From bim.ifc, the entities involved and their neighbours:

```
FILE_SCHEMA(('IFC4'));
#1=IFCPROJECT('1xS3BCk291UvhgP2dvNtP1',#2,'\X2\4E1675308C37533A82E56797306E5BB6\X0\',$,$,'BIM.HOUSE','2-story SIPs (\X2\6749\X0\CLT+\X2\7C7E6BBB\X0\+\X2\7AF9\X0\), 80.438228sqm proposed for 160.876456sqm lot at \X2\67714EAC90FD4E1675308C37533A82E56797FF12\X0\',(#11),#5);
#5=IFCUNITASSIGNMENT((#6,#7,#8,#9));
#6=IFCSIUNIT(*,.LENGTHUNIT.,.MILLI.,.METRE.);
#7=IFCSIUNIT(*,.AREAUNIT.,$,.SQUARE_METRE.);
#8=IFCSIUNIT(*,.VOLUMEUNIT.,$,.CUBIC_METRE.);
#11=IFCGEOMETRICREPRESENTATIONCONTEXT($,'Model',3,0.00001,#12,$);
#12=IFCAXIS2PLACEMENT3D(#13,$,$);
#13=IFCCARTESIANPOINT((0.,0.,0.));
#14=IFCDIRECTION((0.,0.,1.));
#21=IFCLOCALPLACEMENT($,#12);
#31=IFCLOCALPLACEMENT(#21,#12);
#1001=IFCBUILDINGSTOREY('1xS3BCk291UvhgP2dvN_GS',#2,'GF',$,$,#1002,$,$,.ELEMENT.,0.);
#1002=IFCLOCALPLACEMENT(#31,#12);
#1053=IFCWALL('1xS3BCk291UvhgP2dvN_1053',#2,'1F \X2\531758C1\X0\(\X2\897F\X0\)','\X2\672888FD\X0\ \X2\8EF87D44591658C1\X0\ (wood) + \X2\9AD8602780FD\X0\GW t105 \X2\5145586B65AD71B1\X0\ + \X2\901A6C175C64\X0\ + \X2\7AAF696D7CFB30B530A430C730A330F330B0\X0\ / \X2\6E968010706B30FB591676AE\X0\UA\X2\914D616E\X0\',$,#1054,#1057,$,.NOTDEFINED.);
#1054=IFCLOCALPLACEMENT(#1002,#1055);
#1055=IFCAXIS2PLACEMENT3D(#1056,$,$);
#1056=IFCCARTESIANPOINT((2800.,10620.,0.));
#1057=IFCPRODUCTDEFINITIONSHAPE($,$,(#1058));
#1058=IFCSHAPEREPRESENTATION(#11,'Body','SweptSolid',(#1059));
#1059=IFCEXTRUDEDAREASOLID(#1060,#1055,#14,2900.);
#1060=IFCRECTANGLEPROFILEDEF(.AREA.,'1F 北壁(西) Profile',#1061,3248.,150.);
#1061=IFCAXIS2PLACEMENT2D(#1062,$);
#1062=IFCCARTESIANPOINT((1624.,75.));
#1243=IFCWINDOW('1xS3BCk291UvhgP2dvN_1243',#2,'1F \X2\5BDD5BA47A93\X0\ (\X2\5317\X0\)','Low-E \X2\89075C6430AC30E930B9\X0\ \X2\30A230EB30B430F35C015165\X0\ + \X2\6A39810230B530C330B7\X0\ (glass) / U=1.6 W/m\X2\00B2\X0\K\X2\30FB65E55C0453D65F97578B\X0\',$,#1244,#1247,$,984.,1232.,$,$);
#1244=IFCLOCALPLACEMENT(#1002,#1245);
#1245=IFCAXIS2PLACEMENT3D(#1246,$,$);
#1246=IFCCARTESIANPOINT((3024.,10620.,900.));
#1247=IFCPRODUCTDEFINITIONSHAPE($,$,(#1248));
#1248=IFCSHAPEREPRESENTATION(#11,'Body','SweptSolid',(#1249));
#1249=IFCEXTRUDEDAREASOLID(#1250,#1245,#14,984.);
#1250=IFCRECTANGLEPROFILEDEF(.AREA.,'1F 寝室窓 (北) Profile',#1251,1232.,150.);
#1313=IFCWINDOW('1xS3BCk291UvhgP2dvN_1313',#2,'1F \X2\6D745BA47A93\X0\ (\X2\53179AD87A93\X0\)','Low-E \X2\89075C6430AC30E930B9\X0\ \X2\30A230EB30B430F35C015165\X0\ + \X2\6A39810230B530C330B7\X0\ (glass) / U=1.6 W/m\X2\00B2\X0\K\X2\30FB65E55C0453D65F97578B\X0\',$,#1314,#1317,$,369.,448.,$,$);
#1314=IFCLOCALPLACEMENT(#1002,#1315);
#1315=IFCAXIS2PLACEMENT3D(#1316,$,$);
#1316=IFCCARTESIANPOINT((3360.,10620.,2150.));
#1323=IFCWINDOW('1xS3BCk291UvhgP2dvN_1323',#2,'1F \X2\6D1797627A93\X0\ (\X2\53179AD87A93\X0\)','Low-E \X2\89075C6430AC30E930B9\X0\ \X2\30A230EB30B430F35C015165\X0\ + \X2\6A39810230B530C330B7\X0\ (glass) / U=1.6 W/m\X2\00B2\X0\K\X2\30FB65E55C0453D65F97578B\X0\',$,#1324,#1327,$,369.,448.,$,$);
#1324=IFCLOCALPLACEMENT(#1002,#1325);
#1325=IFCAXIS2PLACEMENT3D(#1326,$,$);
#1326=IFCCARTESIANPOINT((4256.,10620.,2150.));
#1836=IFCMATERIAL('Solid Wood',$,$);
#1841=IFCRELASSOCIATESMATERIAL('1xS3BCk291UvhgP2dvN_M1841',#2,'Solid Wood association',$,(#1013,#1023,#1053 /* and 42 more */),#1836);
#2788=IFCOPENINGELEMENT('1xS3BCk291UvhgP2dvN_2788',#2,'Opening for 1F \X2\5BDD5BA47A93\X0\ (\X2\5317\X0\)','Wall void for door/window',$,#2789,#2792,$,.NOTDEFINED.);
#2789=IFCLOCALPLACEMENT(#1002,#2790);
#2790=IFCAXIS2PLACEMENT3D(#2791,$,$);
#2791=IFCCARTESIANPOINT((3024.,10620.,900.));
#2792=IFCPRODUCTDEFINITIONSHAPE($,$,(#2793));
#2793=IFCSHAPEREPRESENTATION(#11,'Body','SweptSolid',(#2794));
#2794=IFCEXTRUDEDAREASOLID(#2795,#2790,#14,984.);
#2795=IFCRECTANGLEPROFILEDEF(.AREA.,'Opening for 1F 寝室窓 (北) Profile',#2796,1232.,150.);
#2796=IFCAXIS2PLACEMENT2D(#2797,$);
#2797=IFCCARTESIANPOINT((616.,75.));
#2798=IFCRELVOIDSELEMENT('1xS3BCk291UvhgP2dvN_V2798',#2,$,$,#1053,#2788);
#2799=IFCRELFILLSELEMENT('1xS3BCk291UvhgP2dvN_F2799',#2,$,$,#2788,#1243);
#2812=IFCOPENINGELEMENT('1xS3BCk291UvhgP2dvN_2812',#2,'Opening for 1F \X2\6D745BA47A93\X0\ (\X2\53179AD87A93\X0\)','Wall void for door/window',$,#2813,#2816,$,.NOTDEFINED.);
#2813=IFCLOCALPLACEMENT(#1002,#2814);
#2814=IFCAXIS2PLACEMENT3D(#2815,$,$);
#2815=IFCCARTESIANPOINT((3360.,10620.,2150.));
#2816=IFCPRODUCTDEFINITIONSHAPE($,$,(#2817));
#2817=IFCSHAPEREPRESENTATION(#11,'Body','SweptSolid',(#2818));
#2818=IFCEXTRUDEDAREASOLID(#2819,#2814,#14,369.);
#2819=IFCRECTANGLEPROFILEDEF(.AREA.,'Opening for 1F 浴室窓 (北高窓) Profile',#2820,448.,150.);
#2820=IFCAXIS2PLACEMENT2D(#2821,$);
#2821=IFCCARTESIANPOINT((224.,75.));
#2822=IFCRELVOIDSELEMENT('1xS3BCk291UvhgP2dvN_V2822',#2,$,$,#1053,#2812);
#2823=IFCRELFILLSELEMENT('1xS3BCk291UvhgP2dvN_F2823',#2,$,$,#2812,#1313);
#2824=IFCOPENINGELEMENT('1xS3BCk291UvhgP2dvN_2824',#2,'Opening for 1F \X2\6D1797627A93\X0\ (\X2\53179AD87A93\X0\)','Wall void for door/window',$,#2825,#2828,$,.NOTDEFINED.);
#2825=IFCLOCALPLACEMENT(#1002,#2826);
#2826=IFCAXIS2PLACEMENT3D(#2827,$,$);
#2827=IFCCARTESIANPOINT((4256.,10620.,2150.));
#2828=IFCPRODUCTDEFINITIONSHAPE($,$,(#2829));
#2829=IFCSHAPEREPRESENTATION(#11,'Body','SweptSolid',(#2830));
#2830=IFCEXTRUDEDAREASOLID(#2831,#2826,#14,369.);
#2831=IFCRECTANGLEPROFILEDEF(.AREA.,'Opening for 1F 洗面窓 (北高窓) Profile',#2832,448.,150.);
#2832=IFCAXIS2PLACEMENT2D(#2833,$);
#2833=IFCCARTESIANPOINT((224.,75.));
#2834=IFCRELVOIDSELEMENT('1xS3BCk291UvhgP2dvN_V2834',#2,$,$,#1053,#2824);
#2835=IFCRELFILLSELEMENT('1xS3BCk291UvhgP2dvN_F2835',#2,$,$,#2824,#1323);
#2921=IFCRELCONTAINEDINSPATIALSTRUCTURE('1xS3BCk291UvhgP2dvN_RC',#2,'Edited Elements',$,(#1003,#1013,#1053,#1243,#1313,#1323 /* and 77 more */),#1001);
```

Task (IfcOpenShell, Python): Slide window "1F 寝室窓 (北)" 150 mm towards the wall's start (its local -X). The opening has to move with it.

```python
import ifcopenshell
import ifcopenshell.api.geometry
import ifcopenshell.util.placement
import ifcopenshell.util.unit

model = ifcopenshell.open("bim.ifc")
unit_scale = ifcopenshell.util.unit.calculate_unit_scale(model)

window = model.by_guid("1xS3BCk291UvhgP2dvN_1243")
opening = window.FillsVoids[0].RelatingOpeningElement
wall = opening.VoidsElements[0].RelatingBuildingElement

wall_matrix = ifcopenshell.util.placement.get_local_placement(wall.ObjectPlacement)
shift = wall_matrix[:3, 0] * -0.15 / unit_scale
before = ifcopenshell.util.placement.get_local_placement(window.ObjectPlacement)[:3, 3].copy()

# The window is not placed relative to its opening, so move both.
for product in (opening, window):
    matrix = ifcopenshell.util.placement.get_local_placement(product.ObjectPlacement)
    matrix[:3, 3] += shift
    ifcopenshell.api.geometry.edit_object_placement(model, product=product, matrix=matrix, is_si=False)

after = ifcopenshell.util.placement.get_local_placement(window.ObjectPlacement)[:3, 3]
print("window moved by", (after - before).round(3) + 0.0)

model.write("bim_rev.ifc")
```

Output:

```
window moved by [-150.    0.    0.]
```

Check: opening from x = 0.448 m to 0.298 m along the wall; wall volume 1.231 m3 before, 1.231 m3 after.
